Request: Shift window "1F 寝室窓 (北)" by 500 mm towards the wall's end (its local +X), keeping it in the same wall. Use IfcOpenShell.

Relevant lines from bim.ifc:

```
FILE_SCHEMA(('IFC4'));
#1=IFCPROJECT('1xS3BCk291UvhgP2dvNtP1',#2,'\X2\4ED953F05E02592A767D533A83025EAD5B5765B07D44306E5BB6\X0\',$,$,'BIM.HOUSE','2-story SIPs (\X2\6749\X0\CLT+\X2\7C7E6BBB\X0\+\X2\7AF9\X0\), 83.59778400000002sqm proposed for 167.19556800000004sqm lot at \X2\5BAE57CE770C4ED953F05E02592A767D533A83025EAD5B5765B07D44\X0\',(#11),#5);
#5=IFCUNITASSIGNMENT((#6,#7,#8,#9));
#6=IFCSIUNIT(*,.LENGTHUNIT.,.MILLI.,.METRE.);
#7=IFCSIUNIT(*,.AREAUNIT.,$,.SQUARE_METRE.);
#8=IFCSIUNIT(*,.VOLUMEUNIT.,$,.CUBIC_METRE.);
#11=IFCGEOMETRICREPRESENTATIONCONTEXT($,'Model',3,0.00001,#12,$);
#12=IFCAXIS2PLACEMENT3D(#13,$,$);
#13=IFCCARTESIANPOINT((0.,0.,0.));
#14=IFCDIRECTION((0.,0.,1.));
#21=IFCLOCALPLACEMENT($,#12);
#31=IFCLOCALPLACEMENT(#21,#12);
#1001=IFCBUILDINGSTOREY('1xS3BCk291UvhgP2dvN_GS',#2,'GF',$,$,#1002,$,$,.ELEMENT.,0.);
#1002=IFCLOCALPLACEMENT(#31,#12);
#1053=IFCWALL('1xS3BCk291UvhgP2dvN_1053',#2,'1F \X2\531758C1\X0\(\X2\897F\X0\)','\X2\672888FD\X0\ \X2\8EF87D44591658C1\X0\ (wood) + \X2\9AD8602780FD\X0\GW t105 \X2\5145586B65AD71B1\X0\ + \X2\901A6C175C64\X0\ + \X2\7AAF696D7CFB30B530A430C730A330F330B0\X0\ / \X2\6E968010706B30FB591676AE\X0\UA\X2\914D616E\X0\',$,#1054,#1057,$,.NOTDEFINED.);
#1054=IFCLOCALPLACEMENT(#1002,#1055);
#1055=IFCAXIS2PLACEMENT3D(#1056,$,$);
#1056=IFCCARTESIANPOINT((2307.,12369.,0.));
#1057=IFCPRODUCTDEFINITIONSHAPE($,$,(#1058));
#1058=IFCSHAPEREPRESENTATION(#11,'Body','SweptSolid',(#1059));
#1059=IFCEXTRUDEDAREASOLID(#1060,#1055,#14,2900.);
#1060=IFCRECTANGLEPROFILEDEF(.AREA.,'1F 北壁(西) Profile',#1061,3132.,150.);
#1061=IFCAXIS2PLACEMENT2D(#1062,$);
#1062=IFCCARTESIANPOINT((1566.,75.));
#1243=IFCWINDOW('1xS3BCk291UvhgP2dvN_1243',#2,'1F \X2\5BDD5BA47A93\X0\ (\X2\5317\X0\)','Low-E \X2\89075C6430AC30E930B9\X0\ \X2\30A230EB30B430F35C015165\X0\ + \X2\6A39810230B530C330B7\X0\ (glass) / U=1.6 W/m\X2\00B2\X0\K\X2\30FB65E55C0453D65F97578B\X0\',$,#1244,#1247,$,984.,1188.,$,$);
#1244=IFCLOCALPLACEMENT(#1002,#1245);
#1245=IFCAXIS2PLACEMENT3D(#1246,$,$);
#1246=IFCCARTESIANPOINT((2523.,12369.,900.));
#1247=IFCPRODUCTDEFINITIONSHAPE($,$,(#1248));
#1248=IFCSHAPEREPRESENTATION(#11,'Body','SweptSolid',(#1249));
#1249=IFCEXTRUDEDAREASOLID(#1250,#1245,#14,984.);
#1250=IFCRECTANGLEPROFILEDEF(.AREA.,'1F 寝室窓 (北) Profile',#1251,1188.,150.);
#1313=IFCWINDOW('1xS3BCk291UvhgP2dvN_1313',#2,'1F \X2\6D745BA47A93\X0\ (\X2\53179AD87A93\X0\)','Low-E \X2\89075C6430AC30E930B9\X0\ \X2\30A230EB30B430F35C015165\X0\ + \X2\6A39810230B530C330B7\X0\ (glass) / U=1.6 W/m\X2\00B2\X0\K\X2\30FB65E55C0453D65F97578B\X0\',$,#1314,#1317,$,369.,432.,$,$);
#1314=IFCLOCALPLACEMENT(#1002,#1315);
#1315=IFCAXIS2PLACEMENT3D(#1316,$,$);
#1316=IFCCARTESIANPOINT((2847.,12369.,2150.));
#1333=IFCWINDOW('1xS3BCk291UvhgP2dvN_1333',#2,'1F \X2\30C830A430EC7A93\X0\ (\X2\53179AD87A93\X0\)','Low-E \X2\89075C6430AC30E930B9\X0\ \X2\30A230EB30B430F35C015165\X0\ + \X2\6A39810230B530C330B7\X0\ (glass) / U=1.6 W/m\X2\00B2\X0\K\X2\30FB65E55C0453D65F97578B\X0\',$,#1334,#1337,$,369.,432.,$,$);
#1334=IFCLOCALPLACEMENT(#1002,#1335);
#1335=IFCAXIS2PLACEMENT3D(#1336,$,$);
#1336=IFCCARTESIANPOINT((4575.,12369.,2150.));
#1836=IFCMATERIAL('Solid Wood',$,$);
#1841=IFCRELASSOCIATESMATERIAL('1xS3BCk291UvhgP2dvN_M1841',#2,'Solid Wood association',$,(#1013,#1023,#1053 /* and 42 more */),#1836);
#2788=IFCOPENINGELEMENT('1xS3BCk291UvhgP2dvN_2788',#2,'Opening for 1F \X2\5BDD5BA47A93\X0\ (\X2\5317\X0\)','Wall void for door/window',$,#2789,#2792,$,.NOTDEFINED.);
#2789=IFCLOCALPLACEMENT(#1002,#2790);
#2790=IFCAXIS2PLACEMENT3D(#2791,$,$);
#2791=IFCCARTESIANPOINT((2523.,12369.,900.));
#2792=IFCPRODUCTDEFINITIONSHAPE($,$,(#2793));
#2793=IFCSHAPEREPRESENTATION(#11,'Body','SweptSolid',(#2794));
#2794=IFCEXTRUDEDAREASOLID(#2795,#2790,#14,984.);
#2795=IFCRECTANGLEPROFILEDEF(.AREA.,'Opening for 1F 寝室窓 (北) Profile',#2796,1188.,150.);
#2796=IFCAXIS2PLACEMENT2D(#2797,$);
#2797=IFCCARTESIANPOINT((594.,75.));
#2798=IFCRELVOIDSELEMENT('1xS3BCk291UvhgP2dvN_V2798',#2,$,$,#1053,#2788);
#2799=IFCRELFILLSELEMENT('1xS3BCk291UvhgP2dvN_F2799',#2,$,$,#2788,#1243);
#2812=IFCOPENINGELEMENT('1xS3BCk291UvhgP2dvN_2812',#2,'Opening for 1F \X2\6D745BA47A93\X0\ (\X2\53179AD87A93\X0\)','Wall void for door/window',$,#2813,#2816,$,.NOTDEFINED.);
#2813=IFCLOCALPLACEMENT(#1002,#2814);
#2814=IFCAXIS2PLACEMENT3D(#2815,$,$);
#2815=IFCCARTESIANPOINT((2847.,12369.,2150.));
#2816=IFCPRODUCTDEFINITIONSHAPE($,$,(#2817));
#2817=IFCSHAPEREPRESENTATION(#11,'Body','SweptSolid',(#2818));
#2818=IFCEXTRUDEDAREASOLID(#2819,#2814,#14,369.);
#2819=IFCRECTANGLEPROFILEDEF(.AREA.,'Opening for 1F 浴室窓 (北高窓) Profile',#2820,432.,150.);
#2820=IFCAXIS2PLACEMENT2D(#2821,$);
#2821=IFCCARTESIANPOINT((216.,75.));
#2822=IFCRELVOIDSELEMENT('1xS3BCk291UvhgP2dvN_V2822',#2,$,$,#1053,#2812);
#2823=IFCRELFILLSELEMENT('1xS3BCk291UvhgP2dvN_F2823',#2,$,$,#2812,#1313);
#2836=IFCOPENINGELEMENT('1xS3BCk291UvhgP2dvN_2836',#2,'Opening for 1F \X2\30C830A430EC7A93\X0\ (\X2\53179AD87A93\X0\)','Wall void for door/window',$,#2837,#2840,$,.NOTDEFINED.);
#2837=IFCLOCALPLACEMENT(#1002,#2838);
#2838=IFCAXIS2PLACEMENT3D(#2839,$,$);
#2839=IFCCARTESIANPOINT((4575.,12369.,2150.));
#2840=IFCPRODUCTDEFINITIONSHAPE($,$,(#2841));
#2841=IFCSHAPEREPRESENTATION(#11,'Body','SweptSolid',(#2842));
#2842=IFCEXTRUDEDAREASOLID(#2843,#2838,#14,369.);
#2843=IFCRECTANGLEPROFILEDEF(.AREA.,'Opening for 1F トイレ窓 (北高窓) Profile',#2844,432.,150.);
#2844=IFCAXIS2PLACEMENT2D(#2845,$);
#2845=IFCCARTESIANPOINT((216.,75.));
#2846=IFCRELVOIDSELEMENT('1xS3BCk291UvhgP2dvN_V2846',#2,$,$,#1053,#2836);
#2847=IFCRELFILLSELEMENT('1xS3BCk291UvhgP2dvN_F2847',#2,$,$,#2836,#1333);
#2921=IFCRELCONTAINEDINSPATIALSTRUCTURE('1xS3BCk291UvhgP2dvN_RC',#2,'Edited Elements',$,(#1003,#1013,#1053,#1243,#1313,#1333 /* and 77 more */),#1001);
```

```python
import ifcopenshell
import ifcopenshell.api.geometry
import ifcopenshell.util.placement
import ifcopenshell.util.unit

model = ifcopenshell.open("bim.ifc")
unit_scale = ifcopenshell.util.unit.calculate_unit_scale(model)

window = model.by_guid("1xS3BCk291UvhgP2dvN_1243")
opening = window.FillsVoids[0].RelatingOpeningElement
wall = opening.VoidsElements[0].RelatingBuildingElement

wall_matrix = ifcopenshell.util.placement.get_local_placement(wall.ObjectPlacement)
shift = wall_matrix[:3, 0] * 0.5 / unit_scale
before = ifcopenshell.util.placement.get_local_placement(window.ObjectPlacement)[:3, 3].copy()

# The window is not placed relative to its opening, so move both.
for product in (opening, window):
    matrix = ifcopenshell.util.placement.get_local_placement(product.ObjectPlacement)
    matrix[:3, 3] += shift
    ifcopenshell.api.geometry.edit_object_placement(model, product=product, matrix=matrix, is_si=False)

after = ifcopenshell.util.placement.get_local_placement(window.ObjectPlacement)[:3, 3]
print("window moved by", (after - before).round(3) + 0.0)

model.write("bim_rev.ifc")
```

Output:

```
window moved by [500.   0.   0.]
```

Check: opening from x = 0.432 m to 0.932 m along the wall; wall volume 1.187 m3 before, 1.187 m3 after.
